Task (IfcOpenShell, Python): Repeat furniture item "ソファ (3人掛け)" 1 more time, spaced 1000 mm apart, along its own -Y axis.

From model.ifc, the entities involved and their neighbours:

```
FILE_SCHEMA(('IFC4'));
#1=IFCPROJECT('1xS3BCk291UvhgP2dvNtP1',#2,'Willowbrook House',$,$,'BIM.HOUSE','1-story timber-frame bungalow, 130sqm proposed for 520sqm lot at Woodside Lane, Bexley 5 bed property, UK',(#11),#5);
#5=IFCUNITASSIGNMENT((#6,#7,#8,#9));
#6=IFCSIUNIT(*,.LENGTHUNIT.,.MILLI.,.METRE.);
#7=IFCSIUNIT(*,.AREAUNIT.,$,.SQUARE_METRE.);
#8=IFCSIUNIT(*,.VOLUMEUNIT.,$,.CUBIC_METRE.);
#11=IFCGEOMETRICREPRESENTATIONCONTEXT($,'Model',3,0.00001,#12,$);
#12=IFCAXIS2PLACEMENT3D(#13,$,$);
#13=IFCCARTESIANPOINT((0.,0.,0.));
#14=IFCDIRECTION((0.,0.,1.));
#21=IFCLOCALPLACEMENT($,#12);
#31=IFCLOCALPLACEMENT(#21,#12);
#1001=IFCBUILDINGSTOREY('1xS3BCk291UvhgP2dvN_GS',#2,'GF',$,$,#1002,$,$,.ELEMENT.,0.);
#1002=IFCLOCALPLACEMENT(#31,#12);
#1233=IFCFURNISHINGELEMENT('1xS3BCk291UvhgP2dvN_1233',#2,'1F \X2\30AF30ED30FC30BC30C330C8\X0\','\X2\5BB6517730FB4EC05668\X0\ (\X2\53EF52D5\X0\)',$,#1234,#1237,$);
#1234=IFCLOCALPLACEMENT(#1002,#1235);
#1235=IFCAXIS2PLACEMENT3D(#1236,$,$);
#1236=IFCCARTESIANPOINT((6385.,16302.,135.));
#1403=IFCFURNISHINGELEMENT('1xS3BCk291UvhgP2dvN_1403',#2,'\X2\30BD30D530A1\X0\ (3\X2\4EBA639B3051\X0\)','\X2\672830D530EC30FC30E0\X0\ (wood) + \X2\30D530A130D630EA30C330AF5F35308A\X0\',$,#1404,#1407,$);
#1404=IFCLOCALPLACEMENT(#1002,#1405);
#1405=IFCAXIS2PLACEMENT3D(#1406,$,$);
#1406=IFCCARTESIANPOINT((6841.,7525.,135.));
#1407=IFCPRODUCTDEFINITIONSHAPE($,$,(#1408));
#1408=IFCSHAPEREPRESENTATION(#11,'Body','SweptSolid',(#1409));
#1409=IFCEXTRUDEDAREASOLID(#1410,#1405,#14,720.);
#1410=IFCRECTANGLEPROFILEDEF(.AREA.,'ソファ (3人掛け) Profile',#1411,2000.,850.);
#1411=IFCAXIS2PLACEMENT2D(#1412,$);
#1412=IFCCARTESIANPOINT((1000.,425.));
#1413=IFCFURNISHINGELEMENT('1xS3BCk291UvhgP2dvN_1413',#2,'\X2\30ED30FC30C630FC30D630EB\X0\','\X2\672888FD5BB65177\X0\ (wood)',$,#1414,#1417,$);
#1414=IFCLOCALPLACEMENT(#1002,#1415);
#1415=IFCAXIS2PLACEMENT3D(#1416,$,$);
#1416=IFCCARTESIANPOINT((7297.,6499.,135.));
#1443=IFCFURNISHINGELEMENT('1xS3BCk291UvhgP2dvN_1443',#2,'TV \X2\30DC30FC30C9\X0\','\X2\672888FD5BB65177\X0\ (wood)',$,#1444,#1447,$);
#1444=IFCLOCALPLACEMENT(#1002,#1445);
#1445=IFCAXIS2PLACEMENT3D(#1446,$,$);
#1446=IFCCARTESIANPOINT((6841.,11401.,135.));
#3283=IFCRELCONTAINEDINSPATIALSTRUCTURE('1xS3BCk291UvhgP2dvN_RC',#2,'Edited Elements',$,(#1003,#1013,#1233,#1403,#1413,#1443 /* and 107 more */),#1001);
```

```python
import ifcopenshell
import ifcopenshell.api.geometry
import ifcopenshell.api.root
import ifcopenshell.util.element
import ifcopenshell.util.placement

model = ifcopenshell.open("model.ifc")


def reuse_history(source, copy):
    """copy_class also copies each property set's owner history, people and application; keep the originals."""
    for rel in copy.IsDefinedBy:
        if rel.is_a("IfcRelDefinesByProperties") and (history := rel.RelatingPropertyDefinition.OwnerHistory):
            rel.RelatingPropertyDefinition.OwnerHistory = source.OwnerHistory
            ifcopenshell.util.element.remove_deep2(model, history)


source = model.by_guid("1xS3BCk291UvhgP2dvN_1403")
base = ifcopenshell.util.placement.get_local_placement(source.ObjectPlacement)
step = -base[:3, 1] * 1000.0

for i in range(1, 2):
    copy = ifcopenshell.api.root.copy_class(model, product=source)
    copy.Representation = ifcopenshell.util.element.copy_deep(
        model, source.Representation, exclude=["IfcGeometricRepresentationContext", "IfcRepresentationMap"]
    )
    reuse_history(source, copy)
    matrix = base.copy()
    matrix[:3, 3] += i * step
    print("added at", matrix[:3, 3].round(3) + 0.0)
    ifcopenshell.api.geometry.edit_object_placement(model, product=copy, matrix=matrix, is_si=False)

model.write("model_updated.ifc")
```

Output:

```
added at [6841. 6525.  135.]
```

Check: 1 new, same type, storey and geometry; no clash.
